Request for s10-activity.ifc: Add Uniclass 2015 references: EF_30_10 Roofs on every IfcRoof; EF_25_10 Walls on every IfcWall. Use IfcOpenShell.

First a look at what the model holds.

```python
import ifcopenshell

model = ifcopenshell.open("s10-activity.ifc")
print(model.schema)
print("classifications:", [c.Name for c in model.by_type("IfcClassification")])
for ifc_class in ("IfcDoor", "IfcRoof", "IfcStair", "IfcWall", "IfcWindow"):
    print(ifc_class, len(model.by_type(ifc_class)))
```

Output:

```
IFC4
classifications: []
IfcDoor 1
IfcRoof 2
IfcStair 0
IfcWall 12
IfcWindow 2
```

```python
import ifcopenshell
import ifcopenshell.api.classification

model = ifcopenshell.open("s10-activity.ifc")

system = ifcopenshell.api.classification.add_classification(model, classification="Uniclass 2015")

codes = {
    "IfcRoof": ("EF_30_10", "Roofs"),
    "IfcWall": ("EF_25_10", "Walls"),
}
for ifc_class, (code, name) in codes.items():
    products = model.by_type(ifc_class)
    ifcopenshell.api.classification.add_reference(
        model, products=products, classification=system, identification=code, name=name
    )
    print(code, len(products))

model.write("s10-activity-out.ifc")
```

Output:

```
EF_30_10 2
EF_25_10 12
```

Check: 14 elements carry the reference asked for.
